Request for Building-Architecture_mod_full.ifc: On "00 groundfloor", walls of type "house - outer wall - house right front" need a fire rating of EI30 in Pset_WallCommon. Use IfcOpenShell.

First a look at what the model holds.

```python
import ifcopenshell
import ifcopenshell.util.element

model = ifcopenshell.open("Building-Architecture_mod_full.ifc")
print(model.schema)
storey = next(s for s in model.by_type("IfcBuildingStorey") if s.Name == "00 groundfloor")
walls = [e for e in ifcopenshell.util.element.get_decomposition(storey) if e.is_a("IfcWall")]
seen = {}
for e in walls:
    element_type = ifcopenshell.util.element.get_type(e)
    key = (element_type.Name if element_type != e and element_type else None, ifcopenshell.util.element.get_pset(e, "Pset_WallCommon", "FireRating"))
    seen[key] = seen.get(key, 0) + 1
for (name, value), count in sorted(seen.items(), key=str):
    print(count, "x", name, "|", value)
```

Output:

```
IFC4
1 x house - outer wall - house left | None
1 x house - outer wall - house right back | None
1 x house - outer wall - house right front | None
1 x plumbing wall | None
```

```python
import ifcopenshell
import ifcopenshell.api.pset
import ifcopenshell.util.element

model = ifcopenshell.open("Building-Architecture_mod_full.ifc")

storey = next(s for s in model.by_type("IfcBuildingStorey") if s.Name == "00 groundfloor")
walls = [e for e in ifcopenshell.util.element.get_decomposition(storey) if e.is_a("IfcWall")]

count = 0
for e in walls:
    element_type = ifcopenshell.util.element.get_type(e)
    if element_type in (None, e) or element_type.Name != "house - outer wall - house right front":
        continue
    # add_pset returns the element's existing set when there is one.
    pset = ifcopenshell.api.pset.add_pset(model, product=e, name="Pset_WallCommon")
    ifcopenshell.api.pset.edit_pset(model, pset=pset, properties={"FireRating": "EI30"})
    count += 1

print(count, "walls updated")

model.write("Building-Architecture_mod_full_edited.ifc")
```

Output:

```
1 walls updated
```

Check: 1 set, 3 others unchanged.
